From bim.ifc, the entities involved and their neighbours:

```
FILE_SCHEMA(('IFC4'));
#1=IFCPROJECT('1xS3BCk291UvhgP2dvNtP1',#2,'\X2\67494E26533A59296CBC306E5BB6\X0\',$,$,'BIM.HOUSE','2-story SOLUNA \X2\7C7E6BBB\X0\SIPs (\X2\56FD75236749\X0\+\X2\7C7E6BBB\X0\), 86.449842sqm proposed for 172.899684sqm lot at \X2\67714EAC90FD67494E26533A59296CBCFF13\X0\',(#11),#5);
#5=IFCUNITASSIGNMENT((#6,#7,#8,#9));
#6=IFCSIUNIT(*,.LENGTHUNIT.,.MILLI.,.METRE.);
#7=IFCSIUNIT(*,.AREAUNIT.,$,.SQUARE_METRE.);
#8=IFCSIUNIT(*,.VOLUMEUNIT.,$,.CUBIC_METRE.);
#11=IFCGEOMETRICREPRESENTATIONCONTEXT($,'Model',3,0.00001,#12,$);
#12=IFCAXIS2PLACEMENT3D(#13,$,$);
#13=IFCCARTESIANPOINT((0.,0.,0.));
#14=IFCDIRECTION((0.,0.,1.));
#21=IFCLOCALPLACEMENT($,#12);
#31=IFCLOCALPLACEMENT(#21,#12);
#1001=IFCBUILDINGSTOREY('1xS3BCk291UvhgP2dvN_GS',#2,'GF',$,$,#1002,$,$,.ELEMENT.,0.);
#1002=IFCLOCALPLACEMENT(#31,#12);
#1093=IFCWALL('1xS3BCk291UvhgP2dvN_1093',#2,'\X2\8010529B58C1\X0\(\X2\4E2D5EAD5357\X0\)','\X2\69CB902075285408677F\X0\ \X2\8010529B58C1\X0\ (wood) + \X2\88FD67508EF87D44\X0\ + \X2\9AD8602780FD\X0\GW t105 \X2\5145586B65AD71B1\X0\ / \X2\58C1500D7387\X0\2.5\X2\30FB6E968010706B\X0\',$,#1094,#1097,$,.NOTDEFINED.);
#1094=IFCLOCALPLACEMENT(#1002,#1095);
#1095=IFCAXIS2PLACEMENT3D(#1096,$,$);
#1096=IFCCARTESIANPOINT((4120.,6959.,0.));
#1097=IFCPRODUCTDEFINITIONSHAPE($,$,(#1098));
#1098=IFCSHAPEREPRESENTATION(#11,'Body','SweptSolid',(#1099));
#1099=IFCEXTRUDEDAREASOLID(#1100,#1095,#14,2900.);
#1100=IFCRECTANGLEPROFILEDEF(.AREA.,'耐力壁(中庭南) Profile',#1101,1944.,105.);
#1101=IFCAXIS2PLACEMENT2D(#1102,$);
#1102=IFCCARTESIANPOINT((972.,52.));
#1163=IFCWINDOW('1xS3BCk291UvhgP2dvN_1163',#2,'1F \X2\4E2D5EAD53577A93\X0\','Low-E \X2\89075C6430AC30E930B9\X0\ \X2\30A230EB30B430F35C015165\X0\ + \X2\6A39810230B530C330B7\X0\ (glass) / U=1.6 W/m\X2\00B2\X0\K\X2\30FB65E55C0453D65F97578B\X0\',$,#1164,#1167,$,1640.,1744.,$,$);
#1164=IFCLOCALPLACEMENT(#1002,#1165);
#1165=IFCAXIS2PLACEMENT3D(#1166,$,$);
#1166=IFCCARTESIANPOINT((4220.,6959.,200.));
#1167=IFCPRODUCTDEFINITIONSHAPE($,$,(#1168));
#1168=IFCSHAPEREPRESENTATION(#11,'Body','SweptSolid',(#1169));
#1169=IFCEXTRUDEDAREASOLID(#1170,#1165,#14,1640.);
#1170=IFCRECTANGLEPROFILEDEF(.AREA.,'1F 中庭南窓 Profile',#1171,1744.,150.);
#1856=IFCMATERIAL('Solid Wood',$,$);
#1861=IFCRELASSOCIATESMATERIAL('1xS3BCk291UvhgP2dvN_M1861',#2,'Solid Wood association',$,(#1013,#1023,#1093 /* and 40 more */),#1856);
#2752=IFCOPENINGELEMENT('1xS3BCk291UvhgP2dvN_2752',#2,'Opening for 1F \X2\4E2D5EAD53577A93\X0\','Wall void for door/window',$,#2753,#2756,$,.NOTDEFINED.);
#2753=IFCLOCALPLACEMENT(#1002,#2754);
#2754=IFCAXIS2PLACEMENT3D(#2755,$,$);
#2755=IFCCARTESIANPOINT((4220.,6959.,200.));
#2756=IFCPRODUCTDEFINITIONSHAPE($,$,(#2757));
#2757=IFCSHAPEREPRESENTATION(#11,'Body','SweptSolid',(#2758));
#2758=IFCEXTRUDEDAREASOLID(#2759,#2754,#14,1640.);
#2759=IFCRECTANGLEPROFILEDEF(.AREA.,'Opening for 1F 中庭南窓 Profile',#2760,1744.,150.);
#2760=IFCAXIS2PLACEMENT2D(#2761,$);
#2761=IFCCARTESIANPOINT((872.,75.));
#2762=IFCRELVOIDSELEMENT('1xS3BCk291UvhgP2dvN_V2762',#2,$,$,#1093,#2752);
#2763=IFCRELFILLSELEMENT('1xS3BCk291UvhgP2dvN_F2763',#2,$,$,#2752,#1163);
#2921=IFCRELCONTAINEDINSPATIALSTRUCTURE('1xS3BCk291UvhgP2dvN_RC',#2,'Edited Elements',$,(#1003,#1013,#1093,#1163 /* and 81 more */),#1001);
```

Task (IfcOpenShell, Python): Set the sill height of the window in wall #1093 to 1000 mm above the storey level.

```python
import numpy as np
import ifcopenshell
import ifcopenshell.api.geometry
import ifcopenshell.geom
import ifcopenshell.util.element
import ifcopenshell.util.placement
import ifcopenshell.util.shape
import ifcopenshell.util.unit

model = ifcopenshell.open("bim.ifc")
unit_scale = ifcopenshell.util.unit.calculate_unit_scale(model)

window = model.by_guid("1xS3BCk291UvhgP2dvN_1163")
opening = window.FillsVoids[0].RelatingOpeningElement
storey = ifcopenshell.util.element.get_container(window, ifc_class="IfcBuildingStorey")
level = ifcopenshell.util.placement.get_local_placement(storey.ObjectPlacement)[2, 3]

# The opening's origin need not be at the sill, so measure its lowest point.
shape = ifcopenshell.geom.create_shape(ifcopenshell.geom.settings(), opening)
bottom = ifcopenshell.util.shape.get_shape_bottom_elevation(shape, shape.geometry) / unit_scale
dz = level + 1 / unit_scale - bottom

shift = np.array([0.0, 0.0, dz])
# The window is not placed relative to its opening, so move both.
for product in (opening, window):
    matrix = ifcopenshell.util.placement.get_local_placement(product.ObjectPlacement)
    matrix[:3, 3] += shift
    ifcopenshell.api.geometry.edit_object_placement(model, product=product, matrix=matrix, is_si=False)

print(f"moved by {dz * unit_scale:+.3f} m")

model.write("bim-out.ifc")
```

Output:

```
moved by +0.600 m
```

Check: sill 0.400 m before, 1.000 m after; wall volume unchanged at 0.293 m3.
